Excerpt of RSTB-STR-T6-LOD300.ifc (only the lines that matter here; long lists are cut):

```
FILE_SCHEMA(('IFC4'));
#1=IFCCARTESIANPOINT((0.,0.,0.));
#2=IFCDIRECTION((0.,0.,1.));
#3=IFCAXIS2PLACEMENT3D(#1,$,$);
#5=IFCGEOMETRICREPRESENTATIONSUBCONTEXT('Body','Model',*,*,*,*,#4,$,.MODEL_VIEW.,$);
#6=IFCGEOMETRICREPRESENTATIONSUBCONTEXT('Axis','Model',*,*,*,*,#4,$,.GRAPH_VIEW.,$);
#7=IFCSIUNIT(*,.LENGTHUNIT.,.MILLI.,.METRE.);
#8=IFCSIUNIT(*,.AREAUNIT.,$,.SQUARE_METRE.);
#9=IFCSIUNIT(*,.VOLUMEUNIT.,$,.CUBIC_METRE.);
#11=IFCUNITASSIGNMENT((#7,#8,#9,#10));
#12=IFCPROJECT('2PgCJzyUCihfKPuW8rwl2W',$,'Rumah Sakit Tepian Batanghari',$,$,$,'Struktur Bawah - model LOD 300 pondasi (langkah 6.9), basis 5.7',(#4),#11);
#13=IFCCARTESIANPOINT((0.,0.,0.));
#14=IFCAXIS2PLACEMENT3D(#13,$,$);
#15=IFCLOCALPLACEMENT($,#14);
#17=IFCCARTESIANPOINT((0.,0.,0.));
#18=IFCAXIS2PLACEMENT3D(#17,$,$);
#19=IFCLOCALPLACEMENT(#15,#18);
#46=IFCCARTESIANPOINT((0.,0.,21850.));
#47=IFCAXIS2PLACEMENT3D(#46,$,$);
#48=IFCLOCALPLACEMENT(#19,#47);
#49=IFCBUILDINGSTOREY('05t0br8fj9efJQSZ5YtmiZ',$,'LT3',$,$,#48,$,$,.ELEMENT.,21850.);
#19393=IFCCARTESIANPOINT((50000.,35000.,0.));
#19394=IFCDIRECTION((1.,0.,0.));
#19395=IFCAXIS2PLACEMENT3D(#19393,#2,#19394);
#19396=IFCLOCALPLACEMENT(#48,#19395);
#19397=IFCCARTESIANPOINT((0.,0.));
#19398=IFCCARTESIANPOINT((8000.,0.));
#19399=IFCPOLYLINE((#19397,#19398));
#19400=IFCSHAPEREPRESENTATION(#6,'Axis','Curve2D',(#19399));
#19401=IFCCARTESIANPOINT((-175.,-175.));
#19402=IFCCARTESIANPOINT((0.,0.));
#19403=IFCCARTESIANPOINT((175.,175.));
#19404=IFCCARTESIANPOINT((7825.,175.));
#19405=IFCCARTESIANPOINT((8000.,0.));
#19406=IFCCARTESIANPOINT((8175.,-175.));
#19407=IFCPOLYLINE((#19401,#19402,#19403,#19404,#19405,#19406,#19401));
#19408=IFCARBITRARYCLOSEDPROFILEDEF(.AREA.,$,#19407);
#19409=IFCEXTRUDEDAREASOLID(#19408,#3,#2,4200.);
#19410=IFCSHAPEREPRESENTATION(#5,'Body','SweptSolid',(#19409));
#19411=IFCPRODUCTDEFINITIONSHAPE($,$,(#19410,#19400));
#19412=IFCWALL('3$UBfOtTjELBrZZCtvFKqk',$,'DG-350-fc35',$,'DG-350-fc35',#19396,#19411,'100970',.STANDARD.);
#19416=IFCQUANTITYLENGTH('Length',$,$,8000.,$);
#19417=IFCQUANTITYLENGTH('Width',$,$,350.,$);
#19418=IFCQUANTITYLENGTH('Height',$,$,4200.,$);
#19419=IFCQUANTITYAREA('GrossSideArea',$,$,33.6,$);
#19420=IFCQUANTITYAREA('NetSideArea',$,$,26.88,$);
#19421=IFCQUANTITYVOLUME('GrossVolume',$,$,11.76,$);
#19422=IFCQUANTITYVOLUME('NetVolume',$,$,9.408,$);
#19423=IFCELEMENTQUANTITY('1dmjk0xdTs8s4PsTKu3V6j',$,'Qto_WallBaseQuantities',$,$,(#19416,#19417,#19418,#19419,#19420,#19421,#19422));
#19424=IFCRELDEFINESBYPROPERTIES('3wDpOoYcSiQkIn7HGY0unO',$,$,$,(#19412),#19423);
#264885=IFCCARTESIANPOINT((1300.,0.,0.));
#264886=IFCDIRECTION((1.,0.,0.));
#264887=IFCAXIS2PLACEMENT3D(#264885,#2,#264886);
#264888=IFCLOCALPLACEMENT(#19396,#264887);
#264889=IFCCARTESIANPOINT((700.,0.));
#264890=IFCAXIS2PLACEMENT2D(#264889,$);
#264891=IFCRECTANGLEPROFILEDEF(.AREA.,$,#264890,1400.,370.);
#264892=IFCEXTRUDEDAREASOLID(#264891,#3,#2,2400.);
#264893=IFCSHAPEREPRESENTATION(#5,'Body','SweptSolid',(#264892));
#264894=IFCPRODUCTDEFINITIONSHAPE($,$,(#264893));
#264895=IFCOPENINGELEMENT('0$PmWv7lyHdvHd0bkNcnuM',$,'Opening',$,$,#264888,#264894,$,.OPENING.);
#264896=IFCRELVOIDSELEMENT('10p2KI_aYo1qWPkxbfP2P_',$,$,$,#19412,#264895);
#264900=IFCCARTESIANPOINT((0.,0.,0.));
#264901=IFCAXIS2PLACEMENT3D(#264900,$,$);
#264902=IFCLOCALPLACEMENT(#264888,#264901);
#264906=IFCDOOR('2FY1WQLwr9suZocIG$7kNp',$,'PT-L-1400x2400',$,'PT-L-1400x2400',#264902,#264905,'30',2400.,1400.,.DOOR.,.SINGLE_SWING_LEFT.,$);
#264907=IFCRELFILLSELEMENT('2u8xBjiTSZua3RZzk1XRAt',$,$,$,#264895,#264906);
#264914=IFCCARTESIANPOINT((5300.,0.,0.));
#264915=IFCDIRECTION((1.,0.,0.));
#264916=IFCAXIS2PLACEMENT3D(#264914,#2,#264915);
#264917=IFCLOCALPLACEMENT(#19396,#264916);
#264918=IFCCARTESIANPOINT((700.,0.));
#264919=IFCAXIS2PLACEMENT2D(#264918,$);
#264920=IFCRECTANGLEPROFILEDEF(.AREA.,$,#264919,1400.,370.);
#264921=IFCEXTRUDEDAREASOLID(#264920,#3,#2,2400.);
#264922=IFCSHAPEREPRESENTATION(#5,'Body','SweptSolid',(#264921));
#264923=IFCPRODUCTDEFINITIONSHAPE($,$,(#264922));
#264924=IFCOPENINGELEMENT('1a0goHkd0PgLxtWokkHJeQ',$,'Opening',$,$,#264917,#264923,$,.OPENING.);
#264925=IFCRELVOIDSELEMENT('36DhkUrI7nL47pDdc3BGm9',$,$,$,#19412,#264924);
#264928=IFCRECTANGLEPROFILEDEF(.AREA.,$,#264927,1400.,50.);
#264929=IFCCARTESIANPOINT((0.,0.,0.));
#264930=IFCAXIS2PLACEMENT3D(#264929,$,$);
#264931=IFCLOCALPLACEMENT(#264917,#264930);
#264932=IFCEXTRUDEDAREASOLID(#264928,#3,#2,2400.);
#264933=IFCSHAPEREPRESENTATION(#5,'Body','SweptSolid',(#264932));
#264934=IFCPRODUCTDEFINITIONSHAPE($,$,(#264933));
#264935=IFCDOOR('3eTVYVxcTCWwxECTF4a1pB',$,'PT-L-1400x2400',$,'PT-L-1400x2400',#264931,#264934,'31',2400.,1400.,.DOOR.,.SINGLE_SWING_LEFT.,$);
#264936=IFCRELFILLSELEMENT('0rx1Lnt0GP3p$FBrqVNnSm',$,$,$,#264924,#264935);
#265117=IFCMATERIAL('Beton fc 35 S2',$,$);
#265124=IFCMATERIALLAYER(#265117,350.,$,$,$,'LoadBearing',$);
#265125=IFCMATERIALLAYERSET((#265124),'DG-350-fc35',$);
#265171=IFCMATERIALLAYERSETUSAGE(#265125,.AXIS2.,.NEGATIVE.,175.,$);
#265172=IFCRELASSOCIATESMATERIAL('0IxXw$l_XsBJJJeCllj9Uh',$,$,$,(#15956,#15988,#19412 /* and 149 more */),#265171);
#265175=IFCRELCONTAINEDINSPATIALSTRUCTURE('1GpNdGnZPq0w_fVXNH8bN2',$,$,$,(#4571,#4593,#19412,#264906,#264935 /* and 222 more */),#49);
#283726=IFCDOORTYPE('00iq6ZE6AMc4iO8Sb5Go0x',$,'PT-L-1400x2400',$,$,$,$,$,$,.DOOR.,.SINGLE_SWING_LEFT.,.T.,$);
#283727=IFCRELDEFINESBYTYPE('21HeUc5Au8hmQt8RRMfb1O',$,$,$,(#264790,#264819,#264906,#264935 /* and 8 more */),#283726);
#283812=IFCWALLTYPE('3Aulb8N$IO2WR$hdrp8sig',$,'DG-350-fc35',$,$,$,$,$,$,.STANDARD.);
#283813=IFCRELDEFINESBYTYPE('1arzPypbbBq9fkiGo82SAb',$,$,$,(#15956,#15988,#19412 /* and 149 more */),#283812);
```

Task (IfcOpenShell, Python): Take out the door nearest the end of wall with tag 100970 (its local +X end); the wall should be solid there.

```python
import ifcopenshell
import ifcopenshell.api.feature
import ifcopenshell.api.pset
import ifcopenshell.api.root
import ifcopenshell.geom
import ifcopenshell.util.element
import ifcopenshell.util.shape
import ifcopenshell.util.unit

model = ifcopenshell.open("RSTB-STR-T6-LOD300.ifc")
area_scale = ifcopenshell.util.unit.calculate_unit_scale(model, "AREAUNIT")
volume_scale = ifcopenshell.util.unit.calculate_unit_scale(model, "VOLUMEUNIT")
settings = ifcopenshell.geom.settings()


def volume(element):
    """Net volume in cubic metres, openings subtracted."""
    shape = ifcopenshell.geom.create_shape(settings, element)
    return ifcopenshell.util.shape.get_volume(shape.geometry)


door = model.by_guid("3eTVYVxcTCWwxECTF4a1pB")
opening = door.FillsVoids[0].RelatingOpeningElement
wall = opening.VoidsElements[0].RelatingBuildingElement
before = volume(wall)

ifcopenshell.api.root.remove_product(model, product=door)
ifcopenshell.api.feature.remove_feature(model, feature=opening)

after = volume(wall)
thickness = 0.35  # wall thickness in metres

# Update the wall's stored quantities.
qto = model.by_id(ifcopenshell.util.element.get_pset(wall, "Qto_WallBaseQuantities", should_inherit=False)["id"])
ifcopenshell.api.pset.edit_qto(model, qto=qto, properties={
    "NetSideArea": after / thickness / area_scale,
    "NetVolume": after / volume_scale,
})

print(f"wall volume {before:.3f} -> {after:.3f} m3")

model.write("RSTB-STR-T6-LOD300_v2.ifc")
```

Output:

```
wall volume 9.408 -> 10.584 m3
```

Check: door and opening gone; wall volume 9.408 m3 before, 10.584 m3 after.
